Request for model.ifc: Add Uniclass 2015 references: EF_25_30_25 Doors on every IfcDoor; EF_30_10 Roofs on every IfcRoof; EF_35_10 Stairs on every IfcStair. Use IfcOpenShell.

First a look at what the model holds.

```python
import ifcopenshell

model = ifcopenshell.open("model.ifc")
print(model.schema)
print("classifications:", [c.Name for c in model.by_type("IfcClassification")])
for ifc_class in ("IfcDoor", "IfcRoof", "IfcStair", "IfcWall", "IfcWindow"):
    print(ifc_class, len(model.by_type(ifc_class)))
```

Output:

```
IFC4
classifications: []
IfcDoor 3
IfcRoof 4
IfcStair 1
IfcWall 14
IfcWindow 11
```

```python
import ifcopenshell
import ifcopenshell.api.classification

model = ifcopenshell.open("model.ifc")

system = ifcopenshell.api.classification.add_classification(model, classification="Uniclass 2015")

codes = {
    "IfcDoor": ("EF_25_30_25", "Doors"),
    "IfcRoof": ("EF_30_10", "Roofs"),
    "IfcStair": ("EF_35_10", "Stairs"),
}
for ifc_class, (code, name) in codes.items():
    products = model.by_type(ifc_class)
    ifcopenshell.api.classification.add_reference(
        model, products=products, classification=system, identification=code, name=name
    )
    print(code, len(products))

model.write("model_rev.ifc")
```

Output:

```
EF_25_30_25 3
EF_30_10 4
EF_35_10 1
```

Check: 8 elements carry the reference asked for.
